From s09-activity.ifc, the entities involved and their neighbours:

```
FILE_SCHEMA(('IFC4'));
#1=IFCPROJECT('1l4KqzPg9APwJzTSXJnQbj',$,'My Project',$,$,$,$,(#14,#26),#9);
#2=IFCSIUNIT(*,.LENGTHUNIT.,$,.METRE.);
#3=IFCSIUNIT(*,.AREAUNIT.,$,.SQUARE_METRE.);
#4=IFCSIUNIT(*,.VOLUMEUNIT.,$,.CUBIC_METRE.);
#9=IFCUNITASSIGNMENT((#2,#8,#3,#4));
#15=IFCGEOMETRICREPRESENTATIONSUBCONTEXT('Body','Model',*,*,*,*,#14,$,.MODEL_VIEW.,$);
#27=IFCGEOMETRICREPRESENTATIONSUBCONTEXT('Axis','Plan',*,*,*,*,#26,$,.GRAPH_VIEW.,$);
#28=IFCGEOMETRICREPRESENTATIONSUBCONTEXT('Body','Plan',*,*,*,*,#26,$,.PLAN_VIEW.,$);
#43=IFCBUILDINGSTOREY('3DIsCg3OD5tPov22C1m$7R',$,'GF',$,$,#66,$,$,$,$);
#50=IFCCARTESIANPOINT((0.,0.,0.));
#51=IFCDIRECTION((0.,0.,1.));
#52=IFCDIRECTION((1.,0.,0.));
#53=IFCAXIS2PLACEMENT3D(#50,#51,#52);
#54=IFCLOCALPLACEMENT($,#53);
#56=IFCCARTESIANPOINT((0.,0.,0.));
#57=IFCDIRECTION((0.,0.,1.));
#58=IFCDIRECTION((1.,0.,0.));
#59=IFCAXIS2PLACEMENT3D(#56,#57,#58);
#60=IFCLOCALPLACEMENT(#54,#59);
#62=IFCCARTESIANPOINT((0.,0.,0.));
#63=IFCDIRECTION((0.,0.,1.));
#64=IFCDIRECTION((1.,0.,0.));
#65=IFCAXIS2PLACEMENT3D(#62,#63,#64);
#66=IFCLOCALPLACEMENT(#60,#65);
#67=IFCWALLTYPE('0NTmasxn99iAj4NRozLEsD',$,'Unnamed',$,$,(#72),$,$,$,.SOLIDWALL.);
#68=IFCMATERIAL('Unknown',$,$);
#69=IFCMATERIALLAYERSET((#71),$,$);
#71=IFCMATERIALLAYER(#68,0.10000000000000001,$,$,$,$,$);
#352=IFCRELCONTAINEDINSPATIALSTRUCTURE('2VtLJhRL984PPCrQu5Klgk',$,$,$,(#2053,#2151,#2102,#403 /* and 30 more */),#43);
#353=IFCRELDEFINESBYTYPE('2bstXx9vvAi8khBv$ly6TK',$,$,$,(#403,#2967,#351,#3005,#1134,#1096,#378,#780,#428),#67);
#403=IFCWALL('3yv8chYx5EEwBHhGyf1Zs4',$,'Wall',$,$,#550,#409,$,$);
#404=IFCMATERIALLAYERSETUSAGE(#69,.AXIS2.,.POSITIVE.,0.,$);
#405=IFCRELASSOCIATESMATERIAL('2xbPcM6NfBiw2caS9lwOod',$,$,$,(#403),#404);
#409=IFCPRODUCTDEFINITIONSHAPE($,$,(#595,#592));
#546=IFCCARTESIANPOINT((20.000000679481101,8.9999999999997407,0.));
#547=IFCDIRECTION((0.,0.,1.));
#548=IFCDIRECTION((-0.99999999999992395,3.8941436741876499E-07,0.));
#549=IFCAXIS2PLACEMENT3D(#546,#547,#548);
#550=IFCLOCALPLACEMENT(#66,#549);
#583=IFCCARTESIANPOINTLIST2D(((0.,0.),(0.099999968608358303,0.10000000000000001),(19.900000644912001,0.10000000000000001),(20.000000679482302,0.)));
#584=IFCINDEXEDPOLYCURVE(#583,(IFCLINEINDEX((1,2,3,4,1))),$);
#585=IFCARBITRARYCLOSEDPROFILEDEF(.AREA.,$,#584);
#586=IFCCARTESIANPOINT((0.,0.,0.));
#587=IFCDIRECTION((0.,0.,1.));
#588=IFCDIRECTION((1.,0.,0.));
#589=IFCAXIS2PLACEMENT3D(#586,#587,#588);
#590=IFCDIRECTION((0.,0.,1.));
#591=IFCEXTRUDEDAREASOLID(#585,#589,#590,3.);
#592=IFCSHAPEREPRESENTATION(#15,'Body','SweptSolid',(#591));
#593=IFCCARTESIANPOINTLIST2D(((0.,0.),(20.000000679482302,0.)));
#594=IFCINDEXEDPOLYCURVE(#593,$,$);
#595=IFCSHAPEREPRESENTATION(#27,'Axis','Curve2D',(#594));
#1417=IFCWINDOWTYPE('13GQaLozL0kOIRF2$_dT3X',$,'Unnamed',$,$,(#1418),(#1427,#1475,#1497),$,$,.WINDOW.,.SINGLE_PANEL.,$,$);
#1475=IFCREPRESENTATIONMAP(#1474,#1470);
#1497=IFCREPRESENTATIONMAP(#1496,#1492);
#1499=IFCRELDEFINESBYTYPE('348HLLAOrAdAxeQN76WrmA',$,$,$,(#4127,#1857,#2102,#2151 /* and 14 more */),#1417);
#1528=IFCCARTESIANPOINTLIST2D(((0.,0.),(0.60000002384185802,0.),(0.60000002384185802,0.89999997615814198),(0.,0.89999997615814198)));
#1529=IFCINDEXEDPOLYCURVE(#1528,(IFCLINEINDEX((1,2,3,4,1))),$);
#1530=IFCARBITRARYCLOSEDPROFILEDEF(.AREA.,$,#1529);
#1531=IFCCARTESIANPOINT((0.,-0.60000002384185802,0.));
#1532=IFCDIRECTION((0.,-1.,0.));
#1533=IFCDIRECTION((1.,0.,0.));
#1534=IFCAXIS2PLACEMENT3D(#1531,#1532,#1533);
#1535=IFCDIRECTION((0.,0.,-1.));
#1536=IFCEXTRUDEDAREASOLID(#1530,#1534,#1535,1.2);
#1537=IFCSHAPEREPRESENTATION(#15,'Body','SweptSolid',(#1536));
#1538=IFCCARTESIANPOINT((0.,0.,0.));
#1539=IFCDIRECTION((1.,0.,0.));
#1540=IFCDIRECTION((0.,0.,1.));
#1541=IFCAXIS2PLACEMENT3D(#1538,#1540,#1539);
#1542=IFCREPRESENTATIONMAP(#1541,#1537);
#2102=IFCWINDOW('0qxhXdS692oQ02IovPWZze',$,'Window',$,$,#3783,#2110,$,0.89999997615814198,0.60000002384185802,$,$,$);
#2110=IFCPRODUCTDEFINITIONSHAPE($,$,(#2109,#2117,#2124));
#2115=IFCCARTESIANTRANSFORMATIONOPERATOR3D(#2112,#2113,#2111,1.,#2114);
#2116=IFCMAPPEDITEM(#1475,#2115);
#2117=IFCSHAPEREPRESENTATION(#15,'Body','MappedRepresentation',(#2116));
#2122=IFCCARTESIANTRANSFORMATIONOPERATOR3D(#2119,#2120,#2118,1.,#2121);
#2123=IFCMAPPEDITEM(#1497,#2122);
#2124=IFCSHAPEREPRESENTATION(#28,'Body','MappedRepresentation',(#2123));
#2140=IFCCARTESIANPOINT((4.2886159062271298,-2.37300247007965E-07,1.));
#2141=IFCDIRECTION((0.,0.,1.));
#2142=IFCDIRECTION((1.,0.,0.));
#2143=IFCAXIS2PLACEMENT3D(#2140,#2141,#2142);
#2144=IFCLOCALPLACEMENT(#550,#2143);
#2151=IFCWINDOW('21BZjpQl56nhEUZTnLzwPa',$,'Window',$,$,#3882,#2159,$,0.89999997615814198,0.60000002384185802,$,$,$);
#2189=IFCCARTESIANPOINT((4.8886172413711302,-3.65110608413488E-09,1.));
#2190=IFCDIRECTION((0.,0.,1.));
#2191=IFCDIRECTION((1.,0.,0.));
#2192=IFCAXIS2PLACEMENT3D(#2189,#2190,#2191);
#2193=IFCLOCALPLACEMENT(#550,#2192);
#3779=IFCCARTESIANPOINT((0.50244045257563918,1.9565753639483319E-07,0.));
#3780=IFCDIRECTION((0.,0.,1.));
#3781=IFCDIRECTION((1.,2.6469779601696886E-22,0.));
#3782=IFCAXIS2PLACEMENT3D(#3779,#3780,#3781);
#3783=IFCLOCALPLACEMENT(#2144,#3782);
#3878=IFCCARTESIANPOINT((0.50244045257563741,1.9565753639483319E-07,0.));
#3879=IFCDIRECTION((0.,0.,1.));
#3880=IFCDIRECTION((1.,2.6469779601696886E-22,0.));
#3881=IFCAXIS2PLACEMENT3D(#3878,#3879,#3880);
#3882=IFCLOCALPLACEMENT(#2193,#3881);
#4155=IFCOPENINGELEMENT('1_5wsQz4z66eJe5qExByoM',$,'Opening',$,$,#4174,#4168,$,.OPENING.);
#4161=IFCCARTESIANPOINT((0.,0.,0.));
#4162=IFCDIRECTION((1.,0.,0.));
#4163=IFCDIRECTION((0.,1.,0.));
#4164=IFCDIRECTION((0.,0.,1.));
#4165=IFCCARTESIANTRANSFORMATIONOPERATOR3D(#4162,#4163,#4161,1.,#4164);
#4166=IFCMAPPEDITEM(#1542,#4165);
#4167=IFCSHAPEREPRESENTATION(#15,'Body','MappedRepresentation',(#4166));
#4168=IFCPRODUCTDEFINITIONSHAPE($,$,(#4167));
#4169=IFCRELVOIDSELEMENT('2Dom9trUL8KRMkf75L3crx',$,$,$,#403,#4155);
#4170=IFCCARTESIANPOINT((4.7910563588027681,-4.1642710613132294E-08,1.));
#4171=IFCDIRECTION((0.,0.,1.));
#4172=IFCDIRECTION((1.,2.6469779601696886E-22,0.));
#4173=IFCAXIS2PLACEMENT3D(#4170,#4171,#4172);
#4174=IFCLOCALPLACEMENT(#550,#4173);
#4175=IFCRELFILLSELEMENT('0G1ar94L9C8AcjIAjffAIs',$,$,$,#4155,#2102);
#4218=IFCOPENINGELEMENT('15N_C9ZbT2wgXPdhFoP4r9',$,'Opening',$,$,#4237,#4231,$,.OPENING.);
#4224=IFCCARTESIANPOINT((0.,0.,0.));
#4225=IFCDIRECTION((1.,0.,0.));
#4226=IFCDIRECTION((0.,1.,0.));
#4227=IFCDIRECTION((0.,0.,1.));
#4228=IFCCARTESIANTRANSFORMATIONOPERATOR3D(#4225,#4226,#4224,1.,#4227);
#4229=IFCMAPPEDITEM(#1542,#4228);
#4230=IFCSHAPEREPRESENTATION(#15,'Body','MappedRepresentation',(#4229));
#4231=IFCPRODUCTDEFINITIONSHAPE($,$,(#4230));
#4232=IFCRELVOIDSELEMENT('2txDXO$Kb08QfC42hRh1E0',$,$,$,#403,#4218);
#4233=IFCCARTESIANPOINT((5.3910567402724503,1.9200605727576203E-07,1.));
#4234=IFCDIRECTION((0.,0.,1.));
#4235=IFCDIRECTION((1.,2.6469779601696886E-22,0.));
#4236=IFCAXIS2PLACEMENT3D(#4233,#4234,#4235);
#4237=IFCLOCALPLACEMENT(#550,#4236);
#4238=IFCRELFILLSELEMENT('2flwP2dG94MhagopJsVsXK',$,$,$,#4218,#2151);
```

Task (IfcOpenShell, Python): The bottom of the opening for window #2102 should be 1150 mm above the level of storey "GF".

```python
import numpy as np
import ifcopenshell
import ifcopenshell.api.geometry
import ifcopenshell.geom
import ifcopenshell.util.element
import ifcopenshell.util.placement
import ifcopenshell.util.shape
import ifcopenshell.util.unit

model = ifcopenshell.open("s09-activity.ifc")
unit_scale = ifcopenshell.util.unit.calculate_unit_scale(model)

window = model.by_id(2102)
opening = window.FillsVoids[0].RelatingOpeningElement
storey = ifcopenshell.util.element.get_container(window, ifc_class="IfcBuildingStorey")
level = ifcopenshell.util.placement.get_local_placement(storey.ObjectPlacement)[2, 3]

# The opening's origin need not be at the sill, so measure its lowest point.
shape = ifcopenshell.geom.create_shape(ifcopenshell.geom.settings(), opening)
bottom = ifcopenshell.util.shape.get_shape_bottom_elevation(shape, shape.geometry) / unit_scale
dz = level + 1.15 - bottom

shift = np.array([0.0, 0.0, dz])
# The window is not placed relative to its opening, so move both.
for product in (opening, window):
    matrix = ifcopenshell.util.placement.get_local_placement(product.ObjectPlacement)
    matrix[:3, 3] += shift
    ifcopenshell.api.geometry.edit_object_placement(model, product=product, matrix=matrix, is_si=False)

print(f"moved by {dz * unit_scale:+.3f} m")

model.write("s09-activity_rev.ifc")
```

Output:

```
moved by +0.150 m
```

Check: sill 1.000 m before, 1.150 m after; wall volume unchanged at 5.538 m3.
